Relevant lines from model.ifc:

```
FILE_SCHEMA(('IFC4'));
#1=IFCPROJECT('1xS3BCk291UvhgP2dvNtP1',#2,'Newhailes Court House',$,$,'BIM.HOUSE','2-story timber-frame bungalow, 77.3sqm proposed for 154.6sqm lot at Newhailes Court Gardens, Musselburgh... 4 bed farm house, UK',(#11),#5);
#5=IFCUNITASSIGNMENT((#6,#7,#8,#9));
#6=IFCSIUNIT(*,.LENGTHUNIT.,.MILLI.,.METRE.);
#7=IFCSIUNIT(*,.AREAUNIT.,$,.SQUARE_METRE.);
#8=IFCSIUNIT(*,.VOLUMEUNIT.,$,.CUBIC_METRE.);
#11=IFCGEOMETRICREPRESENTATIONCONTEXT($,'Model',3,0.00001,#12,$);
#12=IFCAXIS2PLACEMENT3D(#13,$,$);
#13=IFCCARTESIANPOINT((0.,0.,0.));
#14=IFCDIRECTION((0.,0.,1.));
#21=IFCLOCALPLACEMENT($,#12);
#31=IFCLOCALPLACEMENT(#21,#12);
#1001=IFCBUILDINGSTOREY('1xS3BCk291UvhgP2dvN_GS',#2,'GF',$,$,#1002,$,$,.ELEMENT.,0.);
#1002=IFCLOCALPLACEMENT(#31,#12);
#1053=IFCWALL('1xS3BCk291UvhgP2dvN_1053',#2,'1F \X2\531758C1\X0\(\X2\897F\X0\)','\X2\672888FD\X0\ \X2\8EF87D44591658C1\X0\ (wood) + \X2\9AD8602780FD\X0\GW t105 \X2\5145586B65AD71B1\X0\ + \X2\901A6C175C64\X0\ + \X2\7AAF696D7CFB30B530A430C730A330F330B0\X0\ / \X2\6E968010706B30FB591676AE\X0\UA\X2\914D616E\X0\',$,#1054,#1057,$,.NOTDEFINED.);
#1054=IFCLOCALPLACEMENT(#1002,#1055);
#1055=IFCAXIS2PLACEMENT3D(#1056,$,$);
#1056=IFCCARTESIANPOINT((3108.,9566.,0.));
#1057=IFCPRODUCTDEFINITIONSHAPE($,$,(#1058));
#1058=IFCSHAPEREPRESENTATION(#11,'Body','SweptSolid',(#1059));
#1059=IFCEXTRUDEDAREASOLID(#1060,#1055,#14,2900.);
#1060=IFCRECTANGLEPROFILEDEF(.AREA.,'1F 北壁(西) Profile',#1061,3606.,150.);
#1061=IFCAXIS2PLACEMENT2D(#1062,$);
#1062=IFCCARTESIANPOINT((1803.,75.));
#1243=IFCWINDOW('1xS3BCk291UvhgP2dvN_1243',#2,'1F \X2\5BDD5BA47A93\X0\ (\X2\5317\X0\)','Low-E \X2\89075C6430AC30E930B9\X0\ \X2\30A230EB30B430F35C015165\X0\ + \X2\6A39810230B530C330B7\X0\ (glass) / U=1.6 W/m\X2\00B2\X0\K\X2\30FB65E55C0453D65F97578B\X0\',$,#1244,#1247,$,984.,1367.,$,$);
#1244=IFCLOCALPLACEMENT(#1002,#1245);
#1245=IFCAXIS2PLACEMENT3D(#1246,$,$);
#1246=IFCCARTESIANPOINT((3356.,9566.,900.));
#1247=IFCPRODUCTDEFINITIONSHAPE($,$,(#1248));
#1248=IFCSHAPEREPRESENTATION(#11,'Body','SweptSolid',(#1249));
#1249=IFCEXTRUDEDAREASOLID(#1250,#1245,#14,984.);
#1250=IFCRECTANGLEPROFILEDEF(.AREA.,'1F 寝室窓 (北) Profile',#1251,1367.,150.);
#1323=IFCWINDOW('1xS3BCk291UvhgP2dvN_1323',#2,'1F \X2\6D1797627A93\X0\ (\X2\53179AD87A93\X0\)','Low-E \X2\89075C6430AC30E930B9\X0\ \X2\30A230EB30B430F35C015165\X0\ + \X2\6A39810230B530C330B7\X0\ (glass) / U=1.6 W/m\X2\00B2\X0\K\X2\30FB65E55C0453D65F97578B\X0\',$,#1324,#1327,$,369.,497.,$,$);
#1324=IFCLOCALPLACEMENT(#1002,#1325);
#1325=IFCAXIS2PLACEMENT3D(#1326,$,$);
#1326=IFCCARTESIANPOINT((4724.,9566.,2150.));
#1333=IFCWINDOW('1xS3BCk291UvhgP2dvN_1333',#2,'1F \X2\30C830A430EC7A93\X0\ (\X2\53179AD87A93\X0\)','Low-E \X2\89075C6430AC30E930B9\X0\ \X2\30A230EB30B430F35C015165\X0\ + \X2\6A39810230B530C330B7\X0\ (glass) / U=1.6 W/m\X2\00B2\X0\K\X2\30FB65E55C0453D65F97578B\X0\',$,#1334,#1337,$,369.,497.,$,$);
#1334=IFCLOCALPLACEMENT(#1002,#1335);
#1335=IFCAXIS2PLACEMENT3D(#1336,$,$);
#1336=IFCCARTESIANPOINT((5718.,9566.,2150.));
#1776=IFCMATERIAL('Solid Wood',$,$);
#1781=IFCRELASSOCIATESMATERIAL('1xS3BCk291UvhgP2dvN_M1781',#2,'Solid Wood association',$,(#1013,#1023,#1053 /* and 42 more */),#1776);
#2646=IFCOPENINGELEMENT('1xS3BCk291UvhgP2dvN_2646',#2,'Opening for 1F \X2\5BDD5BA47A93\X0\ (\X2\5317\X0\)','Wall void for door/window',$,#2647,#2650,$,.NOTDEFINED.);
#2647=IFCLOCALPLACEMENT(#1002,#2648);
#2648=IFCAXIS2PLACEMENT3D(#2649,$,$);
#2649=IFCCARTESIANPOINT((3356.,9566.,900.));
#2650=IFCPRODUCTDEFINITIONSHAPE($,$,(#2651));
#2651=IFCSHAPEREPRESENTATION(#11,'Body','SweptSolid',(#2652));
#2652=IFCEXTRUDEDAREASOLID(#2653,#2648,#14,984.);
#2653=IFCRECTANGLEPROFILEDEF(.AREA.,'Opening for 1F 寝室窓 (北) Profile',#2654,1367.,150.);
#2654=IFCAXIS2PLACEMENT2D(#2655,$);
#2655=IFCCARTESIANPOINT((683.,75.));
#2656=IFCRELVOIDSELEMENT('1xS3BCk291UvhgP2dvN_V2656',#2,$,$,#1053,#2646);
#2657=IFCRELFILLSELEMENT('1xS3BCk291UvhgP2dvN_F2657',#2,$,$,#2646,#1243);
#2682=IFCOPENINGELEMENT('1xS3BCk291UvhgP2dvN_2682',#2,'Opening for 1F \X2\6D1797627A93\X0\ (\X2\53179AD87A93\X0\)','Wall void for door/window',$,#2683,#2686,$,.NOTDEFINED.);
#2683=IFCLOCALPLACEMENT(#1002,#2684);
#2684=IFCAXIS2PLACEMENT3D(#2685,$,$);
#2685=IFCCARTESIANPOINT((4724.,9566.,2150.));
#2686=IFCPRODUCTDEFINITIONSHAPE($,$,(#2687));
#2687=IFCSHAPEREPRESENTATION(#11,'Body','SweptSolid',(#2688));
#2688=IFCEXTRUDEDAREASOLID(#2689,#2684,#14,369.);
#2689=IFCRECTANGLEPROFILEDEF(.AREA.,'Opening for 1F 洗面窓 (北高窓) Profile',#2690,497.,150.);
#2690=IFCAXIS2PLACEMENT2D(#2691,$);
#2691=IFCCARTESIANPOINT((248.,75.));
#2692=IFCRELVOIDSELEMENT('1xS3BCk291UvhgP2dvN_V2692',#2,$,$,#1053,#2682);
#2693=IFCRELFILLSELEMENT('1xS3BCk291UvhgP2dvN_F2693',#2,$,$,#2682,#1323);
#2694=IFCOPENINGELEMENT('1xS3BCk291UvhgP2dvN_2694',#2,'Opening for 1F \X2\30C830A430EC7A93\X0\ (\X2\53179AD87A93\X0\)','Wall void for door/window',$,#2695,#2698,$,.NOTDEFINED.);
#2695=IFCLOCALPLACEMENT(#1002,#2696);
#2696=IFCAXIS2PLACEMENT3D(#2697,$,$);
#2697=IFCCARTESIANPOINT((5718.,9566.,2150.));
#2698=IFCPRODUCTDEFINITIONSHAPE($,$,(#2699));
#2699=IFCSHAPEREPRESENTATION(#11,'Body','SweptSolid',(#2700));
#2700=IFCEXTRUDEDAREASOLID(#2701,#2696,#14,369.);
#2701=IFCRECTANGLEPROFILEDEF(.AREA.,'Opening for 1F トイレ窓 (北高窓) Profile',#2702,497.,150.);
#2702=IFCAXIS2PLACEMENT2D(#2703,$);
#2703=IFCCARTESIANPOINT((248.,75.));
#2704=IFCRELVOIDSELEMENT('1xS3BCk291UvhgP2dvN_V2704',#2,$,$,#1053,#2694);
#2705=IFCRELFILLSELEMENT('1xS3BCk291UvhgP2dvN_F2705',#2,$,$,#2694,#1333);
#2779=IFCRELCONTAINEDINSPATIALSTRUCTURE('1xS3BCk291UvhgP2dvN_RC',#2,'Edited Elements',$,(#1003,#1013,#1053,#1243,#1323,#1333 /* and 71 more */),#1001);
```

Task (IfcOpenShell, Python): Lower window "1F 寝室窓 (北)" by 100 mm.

```python
import numpy as np
import ifcopenshell
import ifcopenshell.api.geometry
import ifcopenshell.util.placement
import ifcopenshell.util.unit

model = ifcopenshell.open("model.ifc")
unit_scale = ifcopenshell.util.unit.calculate_unit_scale(model)

window = model.by_guid("1xS3BCk291UvhgP2dvN_1243")
opening = window.FillsVoids[0].RelatingOpeningElement
dz = -100.0

shift = np.array([0.0, 0.0, dz])
# The window is not placed relative to its opening, so move both.
for product in (opening, window):
    matrix = ifcopenshell.util.placement.get_local_placement(product.ObjectPlacement)
    matrix[:3, 3] += shift
    ifcopenshell.api.geometry.edit_object_placement(model, product=product, matrix=matrix, is_si=False)

print(f"moved by {dz * unit_scale:+.3f} m")

model.write("model_updated.ifc")
```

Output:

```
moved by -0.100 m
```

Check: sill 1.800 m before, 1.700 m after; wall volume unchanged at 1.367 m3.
